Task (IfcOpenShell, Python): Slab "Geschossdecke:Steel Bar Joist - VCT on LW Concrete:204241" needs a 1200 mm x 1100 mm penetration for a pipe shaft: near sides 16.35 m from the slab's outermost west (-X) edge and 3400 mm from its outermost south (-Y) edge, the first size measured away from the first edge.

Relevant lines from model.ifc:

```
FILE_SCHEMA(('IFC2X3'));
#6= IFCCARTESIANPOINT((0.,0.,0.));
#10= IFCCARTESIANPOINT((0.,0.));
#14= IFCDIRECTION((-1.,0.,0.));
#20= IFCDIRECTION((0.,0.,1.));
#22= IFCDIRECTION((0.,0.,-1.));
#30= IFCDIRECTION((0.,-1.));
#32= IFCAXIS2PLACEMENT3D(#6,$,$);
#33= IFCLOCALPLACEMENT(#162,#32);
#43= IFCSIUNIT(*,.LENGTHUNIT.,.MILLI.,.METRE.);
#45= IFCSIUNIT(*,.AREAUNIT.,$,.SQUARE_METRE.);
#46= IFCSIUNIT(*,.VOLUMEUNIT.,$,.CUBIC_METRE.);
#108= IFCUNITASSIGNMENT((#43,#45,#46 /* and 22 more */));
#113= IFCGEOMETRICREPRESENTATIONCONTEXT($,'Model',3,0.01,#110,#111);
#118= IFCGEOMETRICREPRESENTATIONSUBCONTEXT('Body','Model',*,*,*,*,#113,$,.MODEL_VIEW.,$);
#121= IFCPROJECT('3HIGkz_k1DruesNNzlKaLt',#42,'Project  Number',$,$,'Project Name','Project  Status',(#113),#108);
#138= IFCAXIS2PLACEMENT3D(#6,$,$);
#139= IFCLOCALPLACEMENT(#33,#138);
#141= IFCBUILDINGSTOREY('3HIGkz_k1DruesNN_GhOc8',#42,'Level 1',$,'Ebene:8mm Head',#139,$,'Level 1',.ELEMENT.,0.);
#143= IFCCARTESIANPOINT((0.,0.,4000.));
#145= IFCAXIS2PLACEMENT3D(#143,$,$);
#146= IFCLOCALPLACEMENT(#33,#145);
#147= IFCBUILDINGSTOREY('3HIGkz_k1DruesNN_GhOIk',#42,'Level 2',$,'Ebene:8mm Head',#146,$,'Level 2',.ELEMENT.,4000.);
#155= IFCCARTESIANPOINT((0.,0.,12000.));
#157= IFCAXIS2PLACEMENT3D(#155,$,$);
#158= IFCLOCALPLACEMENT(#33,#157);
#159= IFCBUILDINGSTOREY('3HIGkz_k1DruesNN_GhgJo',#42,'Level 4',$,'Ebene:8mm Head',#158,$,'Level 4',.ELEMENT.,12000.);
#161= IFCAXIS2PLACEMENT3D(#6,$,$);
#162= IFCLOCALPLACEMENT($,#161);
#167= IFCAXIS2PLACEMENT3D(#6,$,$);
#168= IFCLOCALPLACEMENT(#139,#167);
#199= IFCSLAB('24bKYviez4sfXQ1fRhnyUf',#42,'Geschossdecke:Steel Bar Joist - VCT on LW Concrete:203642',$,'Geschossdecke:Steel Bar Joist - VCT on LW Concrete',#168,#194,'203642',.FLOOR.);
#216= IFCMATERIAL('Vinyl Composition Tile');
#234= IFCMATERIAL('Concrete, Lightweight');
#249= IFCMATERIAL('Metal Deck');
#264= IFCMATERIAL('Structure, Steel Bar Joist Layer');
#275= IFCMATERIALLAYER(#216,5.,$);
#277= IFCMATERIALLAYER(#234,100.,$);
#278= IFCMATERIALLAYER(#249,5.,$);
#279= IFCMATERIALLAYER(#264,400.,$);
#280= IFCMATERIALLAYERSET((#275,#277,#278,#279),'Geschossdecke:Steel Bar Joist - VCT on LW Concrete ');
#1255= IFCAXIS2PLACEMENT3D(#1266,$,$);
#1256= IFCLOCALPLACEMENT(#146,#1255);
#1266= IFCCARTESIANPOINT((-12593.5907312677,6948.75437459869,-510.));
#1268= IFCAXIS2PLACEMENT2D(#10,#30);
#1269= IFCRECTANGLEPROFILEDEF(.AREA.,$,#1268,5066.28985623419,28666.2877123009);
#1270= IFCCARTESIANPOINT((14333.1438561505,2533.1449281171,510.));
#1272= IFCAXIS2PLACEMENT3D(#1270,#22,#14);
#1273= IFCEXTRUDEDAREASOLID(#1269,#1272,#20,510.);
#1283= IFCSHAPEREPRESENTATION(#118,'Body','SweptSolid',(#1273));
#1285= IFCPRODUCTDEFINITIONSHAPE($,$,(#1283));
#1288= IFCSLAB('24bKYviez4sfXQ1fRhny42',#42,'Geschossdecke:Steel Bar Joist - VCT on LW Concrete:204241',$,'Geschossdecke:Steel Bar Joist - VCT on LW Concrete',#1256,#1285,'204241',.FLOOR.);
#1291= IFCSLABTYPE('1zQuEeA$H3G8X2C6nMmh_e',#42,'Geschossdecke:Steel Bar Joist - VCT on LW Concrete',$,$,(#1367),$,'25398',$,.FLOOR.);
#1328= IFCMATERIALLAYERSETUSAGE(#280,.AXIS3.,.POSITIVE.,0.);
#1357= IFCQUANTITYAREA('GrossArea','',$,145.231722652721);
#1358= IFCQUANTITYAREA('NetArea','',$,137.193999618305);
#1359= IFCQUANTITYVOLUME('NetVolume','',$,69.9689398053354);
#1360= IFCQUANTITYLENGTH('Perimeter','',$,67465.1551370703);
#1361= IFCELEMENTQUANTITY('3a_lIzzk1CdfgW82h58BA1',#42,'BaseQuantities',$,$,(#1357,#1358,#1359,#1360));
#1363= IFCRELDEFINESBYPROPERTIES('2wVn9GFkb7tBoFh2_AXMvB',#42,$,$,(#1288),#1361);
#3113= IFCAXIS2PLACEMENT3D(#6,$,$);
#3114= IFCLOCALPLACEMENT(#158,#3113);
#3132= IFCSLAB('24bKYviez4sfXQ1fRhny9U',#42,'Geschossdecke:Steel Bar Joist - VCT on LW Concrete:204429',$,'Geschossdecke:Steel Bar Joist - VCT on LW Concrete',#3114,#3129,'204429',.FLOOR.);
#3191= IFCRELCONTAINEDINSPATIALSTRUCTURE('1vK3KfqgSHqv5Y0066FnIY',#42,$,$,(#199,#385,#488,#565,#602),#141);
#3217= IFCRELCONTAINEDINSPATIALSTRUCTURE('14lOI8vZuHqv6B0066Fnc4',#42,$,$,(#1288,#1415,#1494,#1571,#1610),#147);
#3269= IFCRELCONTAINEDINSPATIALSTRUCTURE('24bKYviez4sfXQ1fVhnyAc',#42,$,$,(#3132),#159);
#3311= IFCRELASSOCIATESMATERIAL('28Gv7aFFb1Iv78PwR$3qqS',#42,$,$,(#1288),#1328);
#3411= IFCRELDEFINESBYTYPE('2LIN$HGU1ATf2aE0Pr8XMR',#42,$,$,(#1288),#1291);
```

```python
import numpy as np
import ifcopenshell
import ifcopenshell.api.feature
import ifcopenshell.api.geometry
import ifcopenshell.api.pset
import ifcopenshell.api.root
import ifcopenshell.geom
import ifcopenshell.util.element
import ifcopenshell.util.placement
import ifcopenshell.util.representation
import ifcopenshell.util.shape
import ifcopenshell.util.unit

model = ifcopenshell.open("model.ifc")
unit_scale = ifcopenshell.util.unit.calculate_unit_scale(model)
area_scale = ifcopenshell.util.unit.calculate_unit_scale(model, "AREAUNIT")
volume_scale = ifcopenshell.util.unit.calculate_unit_scale(model, "VOLUMEUNIT")
settings = ifcopenshell.geom.settings()


def volume(element):
    """Net volume in cubic metres, openings subtracted."""
    shape = ifcopenshell.geom.create_shape(settings, element)
    return ifcopenshell.util.shape.get_volume(shape.geometry)


slab = model.by_id(1288)
before = volume(slab)

# Extent in the slab's own axes, in metres. The edges named are its -X and -Y sides.
slab_shape = ifcopenshell.geom.create_shape(settings, slab)
vertices = ifcopenshell.util.shape.get_vertices(slab_shape.geometry)
x_min, y_min, bottom = vertices.min(axis=0)
top = vertices[:, 2].max()

opening = ifcopenshell.api.root.create_entity(model, ifc_class="IfcOpeningElement", name="Pipe shaft opening")
context = ifcopenshell.util.representation.get_context(model, "Model", "Body", "MODEL_VIEW")
width, depth = 1.2, 1.1
outline = [(0.0, 0.0), (width, 0.0), (width, depth), (0.0, depth), (0.0, 0.0)]
# Overshoot both faces by 50 mm so the cut is clean.
shape = ifcopenshell.api.geometry.add_slab_representation(
    model, context=context, depth=top - bottom + 0.1, polyline=outline
)
ifcopenshell.api.geometry.assign_representation(model, product=opening, representation=shape)

matrix = ifcopenshell.util.placement.get_local_placement(slab.ObjectPlacement)
matrix[:, 3] = matrix @ np.append(np.array([x_min + 16.35, y_min + 3.4, bottom - 0.05]) / unit_scale, 1.0)
ifcopenshell.api.geometry.edit_object_placement(model, product=opening, matrix=matrix, is_si=False)
ifcopenshell.api.feature.add_feature(model, feature=opening, element=slab)

after = volume(slab)

# Update the slab's stored quantities.
qto = model.by_id(ifcopenshell.util.element.get_pset(slab, "BaseQuantities", should_inherit=False)["id"])
ifcopenshell.api.pset.edit_qto(model, qto=qto, properties={
    "NetArea": after / (top - bottom) / area_scale,
    "NetVolume": after / volume_scale,
})

print(f"slab volume {before:.3f} -> {after:.3f} m3")

model.write("model_rev.ifc")
```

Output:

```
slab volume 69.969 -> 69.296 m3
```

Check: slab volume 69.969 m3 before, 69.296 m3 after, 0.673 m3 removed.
